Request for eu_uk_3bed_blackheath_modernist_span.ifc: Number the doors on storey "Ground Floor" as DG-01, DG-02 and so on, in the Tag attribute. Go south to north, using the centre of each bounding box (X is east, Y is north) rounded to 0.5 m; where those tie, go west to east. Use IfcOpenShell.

First a look at what the model holds.

```python
import ifcopenshell
import ifcopenshell.util.element
import ifcopenshell.util.placement

model = ifcopenshell.open("eu_uk_3bed_blackheath_modernist_span.ifc")
print(model.schema)
storey = next(s for s in model.by_type("IfcBuildingStorey") if s.Name == "Ground Floor")
doors = [e for e in ifcopenshell.util.element.get_decomposition(storey) if e.is_a("IfcDoor")]
for e in sorted(doors, key=lambda e: e.id()):
    origin = ifcopenshell.util.placement.get_local_placement(e.ObjectPlacement)[:3, 3]
    print(e.id(), e.Tag, e.Name, origin.round(2) + 0.0, sep=" | ")
```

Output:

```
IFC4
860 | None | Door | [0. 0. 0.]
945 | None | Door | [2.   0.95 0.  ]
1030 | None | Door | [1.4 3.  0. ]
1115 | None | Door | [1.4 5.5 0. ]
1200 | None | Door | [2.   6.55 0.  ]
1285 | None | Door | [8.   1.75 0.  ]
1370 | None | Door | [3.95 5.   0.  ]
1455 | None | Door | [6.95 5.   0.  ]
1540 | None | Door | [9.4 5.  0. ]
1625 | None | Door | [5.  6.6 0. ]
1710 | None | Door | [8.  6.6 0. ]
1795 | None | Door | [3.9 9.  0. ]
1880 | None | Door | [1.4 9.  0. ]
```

```python
import ifcopenshell
import ifcopenshell.geom
import ifcopenshell.util.element
import ifcopenshell.util.shape

model = ifcopenshell.open("eu_uk_3bed_blackheath_modernist_span.ifc")
settings = ifcopenshell.geom.settings()
settings.set("use-world-coords", True)


def centre(element):
    shape = ifcopenshell.geom.create_shape(settings, element)
    return ifcopenshell.util.shape.get_bbox_centroid(shape.geometry)


storey = next(s for s in model.by_type("IfcBuildingStorey") if s.Name == "Ground Floor")
doors = [e for e in ifcopenshell.util.element.get_decomposition(storey) if e.is_a("IfcDoor")]

# Insertion points can sit at a corner or the storey origin, so sort by the geometry (in metres).
centres = {e: centre(e) for e in doors}
doors.sort(key=lambda e: (round(centres[e][1] / 0.5), centres[e][0]))

for i, e in enumerate(doors, start=1):
    number = f"DG-{i:02d}"
    e.Tag = number
    print(e.id(), number)

model.write("eu_uk_3bed_blackheath_modernist_span-out.ifc")
```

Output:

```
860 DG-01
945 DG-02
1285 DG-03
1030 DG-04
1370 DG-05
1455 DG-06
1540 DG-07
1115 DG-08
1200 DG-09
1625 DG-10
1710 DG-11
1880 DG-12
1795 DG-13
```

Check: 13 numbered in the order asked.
